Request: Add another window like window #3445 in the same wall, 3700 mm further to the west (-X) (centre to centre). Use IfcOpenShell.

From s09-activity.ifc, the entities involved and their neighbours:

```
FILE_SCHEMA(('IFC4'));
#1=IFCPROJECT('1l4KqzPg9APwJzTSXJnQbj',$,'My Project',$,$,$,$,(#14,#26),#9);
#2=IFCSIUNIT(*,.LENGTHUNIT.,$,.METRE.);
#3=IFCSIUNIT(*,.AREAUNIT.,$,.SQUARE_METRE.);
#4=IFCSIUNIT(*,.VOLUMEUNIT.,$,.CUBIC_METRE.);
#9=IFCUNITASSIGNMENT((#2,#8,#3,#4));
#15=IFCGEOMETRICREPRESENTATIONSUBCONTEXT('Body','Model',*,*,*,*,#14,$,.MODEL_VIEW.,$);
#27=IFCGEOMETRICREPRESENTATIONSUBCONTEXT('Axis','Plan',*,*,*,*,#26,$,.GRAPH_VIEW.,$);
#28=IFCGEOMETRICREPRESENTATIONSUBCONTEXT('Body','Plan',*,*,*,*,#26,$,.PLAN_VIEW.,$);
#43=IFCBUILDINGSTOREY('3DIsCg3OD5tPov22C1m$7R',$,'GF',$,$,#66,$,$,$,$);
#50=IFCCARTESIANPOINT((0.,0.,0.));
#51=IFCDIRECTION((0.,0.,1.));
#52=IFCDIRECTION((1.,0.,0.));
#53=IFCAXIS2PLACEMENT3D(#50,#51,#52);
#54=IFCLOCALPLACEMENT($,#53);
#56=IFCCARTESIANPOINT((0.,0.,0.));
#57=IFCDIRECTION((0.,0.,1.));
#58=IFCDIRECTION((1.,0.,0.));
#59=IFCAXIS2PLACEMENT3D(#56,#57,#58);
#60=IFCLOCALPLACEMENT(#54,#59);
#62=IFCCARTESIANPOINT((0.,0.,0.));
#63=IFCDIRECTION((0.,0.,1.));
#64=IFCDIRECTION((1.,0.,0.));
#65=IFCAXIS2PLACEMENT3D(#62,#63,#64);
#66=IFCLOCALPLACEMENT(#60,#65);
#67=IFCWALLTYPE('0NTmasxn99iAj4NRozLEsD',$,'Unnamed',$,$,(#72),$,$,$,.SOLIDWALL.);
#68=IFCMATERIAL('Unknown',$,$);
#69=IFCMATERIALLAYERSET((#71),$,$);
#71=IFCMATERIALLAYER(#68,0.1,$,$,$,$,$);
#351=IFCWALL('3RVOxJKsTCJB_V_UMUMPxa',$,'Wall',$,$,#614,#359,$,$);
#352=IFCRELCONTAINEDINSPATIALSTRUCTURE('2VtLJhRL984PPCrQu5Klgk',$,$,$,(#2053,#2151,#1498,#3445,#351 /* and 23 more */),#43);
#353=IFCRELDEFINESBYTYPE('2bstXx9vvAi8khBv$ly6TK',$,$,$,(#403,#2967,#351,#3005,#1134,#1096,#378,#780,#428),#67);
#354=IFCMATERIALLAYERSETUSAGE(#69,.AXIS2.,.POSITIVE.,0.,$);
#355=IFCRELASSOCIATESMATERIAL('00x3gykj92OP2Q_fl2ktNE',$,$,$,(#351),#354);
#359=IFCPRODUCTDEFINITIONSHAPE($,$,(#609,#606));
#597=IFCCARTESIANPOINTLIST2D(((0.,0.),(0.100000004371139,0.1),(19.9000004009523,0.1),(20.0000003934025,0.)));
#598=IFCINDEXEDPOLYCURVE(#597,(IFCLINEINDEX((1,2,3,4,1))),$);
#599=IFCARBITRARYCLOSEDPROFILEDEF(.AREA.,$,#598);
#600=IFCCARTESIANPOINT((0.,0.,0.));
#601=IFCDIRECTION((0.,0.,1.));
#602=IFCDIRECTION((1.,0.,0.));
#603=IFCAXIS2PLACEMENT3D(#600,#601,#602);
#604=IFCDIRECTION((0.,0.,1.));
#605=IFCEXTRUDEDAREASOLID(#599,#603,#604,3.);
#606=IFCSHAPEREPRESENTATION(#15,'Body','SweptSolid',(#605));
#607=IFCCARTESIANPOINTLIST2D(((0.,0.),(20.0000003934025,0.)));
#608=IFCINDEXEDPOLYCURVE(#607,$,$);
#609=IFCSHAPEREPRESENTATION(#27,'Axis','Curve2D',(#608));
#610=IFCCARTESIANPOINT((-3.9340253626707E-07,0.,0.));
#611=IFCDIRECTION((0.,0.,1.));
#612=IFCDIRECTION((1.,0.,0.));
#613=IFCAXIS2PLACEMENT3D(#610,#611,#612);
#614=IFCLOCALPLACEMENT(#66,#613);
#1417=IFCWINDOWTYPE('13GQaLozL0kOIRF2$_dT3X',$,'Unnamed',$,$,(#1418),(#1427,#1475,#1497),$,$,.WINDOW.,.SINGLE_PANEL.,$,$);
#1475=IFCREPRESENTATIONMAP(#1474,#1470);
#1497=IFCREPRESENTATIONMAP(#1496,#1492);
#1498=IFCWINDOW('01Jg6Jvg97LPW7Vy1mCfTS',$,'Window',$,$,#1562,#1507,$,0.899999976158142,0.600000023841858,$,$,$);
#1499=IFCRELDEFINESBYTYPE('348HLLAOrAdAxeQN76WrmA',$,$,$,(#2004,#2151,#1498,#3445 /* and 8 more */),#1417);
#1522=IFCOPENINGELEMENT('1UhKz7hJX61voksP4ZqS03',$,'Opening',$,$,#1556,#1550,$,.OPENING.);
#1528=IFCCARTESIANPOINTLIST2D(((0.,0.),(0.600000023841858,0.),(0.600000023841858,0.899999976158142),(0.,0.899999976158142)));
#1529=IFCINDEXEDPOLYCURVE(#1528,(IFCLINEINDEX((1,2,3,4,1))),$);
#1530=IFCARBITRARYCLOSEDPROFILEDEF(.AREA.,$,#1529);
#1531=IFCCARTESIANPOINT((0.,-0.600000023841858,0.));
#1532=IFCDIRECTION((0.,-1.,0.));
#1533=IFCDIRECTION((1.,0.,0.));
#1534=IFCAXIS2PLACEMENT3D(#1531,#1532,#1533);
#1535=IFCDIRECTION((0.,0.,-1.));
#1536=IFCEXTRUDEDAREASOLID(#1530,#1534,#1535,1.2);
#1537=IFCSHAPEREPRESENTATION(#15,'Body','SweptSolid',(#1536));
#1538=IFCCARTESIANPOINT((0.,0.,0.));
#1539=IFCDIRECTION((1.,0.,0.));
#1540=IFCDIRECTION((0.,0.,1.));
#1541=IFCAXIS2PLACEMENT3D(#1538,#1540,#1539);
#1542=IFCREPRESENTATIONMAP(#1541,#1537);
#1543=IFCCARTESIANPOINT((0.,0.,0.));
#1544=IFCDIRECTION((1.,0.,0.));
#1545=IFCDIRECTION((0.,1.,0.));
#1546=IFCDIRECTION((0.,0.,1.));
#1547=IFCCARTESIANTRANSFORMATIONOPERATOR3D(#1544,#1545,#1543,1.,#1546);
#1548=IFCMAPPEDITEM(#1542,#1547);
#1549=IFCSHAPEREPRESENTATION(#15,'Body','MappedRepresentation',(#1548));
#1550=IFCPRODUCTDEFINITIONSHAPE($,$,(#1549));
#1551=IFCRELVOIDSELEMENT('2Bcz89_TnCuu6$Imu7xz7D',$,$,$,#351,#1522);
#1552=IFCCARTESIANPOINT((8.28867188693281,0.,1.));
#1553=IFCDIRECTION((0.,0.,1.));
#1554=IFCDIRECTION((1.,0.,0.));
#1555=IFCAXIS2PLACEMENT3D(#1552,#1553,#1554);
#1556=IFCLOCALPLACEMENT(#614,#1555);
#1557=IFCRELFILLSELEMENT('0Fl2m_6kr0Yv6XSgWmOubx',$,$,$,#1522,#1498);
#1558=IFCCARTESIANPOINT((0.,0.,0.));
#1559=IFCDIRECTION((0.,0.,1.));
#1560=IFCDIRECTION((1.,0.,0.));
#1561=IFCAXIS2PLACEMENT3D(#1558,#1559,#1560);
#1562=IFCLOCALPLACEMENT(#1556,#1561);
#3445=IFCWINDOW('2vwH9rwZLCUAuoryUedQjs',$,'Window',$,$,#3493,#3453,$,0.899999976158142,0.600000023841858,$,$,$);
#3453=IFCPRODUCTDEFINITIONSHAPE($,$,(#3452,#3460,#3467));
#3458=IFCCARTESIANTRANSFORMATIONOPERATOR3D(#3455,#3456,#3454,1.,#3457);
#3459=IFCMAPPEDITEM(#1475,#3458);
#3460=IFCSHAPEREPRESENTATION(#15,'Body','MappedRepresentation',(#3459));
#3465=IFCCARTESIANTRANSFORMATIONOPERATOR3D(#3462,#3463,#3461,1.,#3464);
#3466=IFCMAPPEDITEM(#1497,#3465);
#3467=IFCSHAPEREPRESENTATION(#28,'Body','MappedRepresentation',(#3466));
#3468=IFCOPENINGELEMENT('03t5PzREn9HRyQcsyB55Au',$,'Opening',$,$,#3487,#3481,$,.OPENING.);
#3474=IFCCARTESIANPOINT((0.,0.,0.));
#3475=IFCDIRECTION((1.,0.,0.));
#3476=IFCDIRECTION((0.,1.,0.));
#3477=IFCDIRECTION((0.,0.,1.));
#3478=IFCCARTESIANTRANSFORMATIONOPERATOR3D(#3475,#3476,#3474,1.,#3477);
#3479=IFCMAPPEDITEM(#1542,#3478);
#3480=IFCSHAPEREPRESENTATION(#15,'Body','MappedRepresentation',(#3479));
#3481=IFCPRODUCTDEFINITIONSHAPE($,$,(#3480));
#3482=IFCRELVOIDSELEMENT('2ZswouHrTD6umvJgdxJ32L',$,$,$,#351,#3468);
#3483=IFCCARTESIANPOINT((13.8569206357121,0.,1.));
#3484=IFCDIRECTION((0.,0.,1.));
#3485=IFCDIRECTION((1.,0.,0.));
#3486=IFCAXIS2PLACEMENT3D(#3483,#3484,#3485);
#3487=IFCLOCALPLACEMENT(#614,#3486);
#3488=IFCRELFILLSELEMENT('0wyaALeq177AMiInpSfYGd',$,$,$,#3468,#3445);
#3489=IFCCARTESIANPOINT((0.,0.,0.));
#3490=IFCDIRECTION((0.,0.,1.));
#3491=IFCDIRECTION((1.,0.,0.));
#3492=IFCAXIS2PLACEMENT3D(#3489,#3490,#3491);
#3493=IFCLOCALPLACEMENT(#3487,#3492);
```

```python
import ifcopenshell
import ifcopenshell.api.feature
import ifcopenshell.api.geometry
import ifcopenshell.api.root
import ifcopenshell.geom
import ifcopenshell.util.element
import ifcopenshell.util.placement
import ifcopenshell.util.shape
import ifcopenshell.util.unit

model = ifcopenshell.open("s09-activity.ifc")
unit_scale = ifcopenshell.util.unit.calculate_unit_scale(model)
settings = ifcopenshell.geom.settings()


def volume(element):
    """Net volume in cubic metres, openings subtracted."""
    shape = ifcopenshell.geom.create_shape(settings, element)
    return ifcopenshell.util.shape.get_volume(shape.geometry)


window = model.by_guid("2vwH9rwZLCUAuoryUedQjs")
opening = window.FillsVoids[0].RelatingOpeningElement
wall = opening.VoidsElements[0].RelatingBuildingElement
before = volume(wall)
shift = ifcopenshell.util.placement.get_local_placement(wall.ObjectPlacement)[:3, 0] * -3.7 / unit_scale

# copy_class copies the void relationship, type, container and properties, but no geometry.
new_opening = ifcopenshell.api.root.copy_class(model, product=opening)
new_opening.Representation = ifcopenshell.util.element.copy_deep(
    model, opening.Representation, exclude=["IfcGeometricRepresentationContext", "IfcRepresentationMap"]
)
new_window = ifcopenshell.api.root.copy_class(model, product=window)
new_window.Representation = ifcopenshell.util.element.copy_deep(
    model, window.Representation, exclude=["IfcGeometricRepresentationContext", "IfcRepresentationMap"]
)
ifcopenshell.api.feature.add_filling(model, opening=new_opening, element=new_window)

for old, new in ((opening, new_opening), (window, new_window)):
    matrix = ifcopenshell.util.placement.get_local_placement(old.ObjectPlacement)
    matrix[:3, 3] += shift
    ifcopenshell.api.geometry.edit_object_placement(model, product=new, matrix=matrix, is_si=False)

after = volume(wall)

print(f"wall volume {before:.3f} -> {after:.3f} m3")

model.write("s09-activity_rev.ifc")
```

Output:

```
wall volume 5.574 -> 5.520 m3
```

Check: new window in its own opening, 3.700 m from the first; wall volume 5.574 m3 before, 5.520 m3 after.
